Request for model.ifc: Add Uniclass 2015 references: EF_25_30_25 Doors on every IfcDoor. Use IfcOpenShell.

First a look at what the model holds.

```python
import ifcopenshell

model = ifcopenshell.open("model.ifc")
print(model.schema)
print("classifications:", [c.Name for c in model.by_type("IfcClassification")])
for ifc_class in ("IfcDoor", "IfcRoof", "IfcStair", "IfcWall", "IfcWindow"):
    print(ifc_class, len(model.by_type(ifc_class)))
```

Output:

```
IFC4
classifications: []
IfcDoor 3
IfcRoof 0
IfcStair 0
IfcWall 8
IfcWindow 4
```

```python
import ifcopenshell
import ifcopenshell.api.classification

model = ifcopenshell.open("model.ifc")

system = ifcopenshell.api.classification.add_classification(model, classification="Uniclass 2015")

codes = {
    "IfcDoor": ("EF_25_30_25", "Doors"),
}
for ifc_class, (code, name) in codes.items():
    products = model.by_type(ifc_class)
    ifcopenshell.api.classification.add_reference(
        model, products=products, classification=system, identification=code, name=name
    )
    print(code, len(products))

model.write("model-out.ifc")
```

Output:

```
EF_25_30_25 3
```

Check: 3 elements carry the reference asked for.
